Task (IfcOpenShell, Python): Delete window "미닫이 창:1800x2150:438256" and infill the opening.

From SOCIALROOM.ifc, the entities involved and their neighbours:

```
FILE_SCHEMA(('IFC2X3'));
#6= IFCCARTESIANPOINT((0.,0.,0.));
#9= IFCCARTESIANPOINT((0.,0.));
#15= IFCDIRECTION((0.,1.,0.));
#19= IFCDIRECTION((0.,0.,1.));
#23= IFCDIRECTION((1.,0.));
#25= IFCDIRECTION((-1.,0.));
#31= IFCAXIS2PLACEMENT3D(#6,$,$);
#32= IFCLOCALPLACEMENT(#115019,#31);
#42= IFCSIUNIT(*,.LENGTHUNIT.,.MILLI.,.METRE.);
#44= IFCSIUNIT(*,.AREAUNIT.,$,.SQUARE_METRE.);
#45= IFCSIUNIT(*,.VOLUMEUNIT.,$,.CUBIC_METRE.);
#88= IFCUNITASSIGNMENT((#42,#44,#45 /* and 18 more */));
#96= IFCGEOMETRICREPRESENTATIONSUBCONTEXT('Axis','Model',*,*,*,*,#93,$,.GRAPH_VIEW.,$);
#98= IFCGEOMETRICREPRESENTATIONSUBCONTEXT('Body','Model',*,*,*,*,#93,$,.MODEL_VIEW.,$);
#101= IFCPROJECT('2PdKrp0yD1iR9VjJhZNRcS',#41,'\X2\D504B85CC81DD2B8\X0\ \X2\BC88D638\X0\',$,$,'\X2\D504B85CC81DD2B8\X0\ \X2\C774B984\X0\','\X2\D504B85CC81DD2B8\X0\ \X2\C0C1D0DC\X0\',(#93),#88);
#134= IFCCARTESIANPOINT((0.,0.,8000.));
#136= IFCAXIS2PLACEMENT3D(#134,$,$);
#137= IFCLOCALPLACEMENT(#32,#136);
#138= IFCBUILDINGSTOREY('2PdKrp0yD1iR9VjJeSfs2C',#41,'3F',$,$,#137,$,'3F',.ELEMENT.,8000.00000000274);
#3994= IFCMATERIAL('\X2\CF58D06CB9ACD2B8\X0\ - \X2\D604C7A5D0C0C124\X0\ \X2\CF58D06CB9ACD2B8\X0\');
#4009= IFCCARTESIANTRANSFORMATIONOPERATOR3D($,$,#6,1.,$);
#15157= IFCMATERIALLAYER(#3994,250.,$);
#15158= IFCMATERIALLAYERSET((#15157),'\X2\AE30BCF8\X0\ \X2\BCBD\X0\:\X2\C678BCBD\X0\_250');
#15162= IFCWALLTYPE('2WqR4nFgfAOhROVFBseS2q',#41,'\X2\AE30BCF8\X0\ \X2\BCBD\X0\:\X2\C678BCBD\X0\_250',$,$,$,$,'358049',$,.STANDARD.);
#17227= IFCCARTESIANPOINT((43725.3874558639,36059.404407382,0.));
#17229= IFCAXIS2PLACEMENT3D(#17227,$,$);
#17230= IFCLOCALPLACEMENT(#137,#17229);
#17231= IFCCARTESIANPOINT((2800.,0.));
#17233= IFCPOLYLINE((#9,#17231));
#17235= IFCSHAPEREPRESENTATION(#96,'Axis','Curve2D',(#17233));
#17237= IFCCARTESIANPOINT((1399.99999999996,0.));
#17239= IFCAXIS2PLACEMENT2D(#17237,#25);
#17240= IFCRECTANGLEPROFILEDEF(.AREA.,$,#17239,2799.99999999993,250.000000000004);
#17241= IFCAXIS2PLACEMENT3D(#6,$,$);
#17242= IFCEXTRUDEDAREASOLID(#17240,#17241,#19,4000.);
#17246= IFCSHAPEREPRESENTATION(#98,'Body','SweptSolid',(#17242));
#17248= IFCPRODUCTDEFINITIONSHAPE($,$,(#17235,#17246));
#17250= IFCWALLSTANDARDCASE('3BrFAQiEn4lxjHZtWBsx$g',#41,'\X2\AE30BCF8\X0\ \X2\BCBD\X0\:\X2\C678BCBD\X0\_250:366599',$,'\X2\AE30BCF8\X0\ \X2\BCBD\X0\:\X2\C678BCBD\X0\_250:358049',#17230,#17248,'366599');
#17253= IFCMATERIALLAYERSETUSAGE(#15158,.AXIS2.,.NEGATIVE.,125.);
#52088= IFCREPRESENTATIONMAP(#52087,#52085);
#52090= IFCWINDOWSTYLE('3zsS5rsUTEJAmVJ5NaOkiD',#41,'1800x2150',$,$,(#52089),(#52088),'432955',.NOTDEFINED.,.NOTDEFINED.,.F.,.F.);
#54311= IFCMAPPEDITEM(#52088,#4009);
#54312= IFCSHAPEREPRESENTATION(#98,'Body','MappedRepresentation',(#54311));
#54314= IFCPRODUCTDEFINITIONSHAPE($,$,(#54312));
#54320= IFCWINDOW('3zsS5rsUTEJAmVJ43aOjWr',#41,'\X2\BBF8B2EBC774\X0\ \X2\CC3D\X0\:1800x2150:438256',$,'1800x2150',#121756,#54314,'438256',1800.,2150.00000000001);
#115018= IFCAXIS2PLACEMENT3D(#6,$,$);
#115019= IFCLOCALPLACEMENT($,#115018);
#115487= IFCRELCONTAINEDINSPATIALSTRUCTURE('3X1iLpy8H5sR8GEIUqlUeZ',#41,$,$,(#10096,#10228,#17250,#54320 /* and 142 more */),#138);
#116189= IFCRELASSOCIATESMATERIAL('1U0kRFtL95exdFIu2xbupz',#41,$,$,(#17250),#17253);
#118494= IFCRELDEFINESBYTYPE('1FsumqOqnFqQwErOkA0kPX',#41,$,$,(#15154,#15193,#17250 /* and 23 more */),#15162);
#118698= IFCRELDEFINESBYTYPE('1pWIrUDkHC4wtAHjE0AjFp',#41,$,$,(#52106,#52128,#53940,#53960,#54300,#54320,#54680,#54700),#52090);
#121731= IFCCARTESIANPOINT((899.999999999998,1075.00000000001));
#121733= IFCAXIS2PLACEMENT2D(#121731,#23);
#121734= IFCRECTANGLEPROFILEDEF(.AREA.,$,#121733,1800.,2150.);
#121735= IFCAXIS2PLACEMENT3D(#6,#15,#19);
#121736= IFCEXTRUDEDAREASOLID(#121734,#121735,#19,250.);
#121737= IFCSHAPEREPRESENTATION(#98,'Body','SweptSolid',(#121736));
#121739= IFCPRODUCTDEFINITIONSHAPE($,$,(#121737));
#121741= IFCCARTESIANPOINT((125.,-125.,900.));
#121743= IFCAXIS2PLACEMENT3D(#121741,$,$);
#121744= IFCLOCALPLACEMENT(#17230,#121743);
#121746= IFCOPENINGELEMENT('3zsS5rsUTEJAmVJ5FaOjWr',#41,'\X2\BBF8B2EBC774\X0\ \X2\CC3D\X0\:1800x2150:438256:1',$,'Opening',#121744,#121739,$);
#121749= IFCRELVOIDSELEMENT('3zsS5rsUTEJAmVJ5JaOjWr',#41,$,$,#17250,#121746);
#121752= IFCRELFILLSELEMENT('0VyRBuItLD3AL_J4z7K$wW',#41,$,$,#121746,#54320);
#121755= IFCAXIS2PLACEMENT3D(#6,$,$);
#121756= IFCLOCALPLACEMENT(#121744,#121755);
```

```python
import ifcopenshell
import ifcopenshell.api.feature
import ifcopenshell.api.root
import ifcopenshell.geom
import ifcopenshell.util.shape

model = ifcopenshell.open("SOCIALROOM.ifc")
settings = ifcopenshell.geom.settings()


def volume(element):
    """Net volume in cubic metres, openings subtracted."""
    shape = ifcopenshell.geom.create_shape(settings, element)
    return ifcopenshell.util.shape.get_volume(shape.geometry)


window = model.by_id(54320)
opening = window.FillsVoids[0].RelatingOpeningElement
wall = opening.VoidsElements[0].RelatingBuildingElement
before = volume(wall)

ifcopenshell.api.root.remove_product(model, product=window)
ifcopenshell.api.feature.remove_feature(model, feature=opening)

after = volume(wall)

print(f"wall volume {before:.3f} -> {after:.3f} m3")

model.write("SOCIALROOM_updated.ifc")
```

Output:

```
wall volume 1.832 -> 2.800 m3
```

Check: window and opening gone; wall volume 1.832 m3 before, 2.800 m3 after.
